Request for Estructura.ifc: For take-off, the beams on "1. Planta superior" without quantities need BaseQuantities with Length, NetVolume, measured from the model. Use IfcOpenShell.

First a look at what the model holds.

```python
import ifcopenshell
import ifcopenshell.util.element
import ifcopenshell.util.unit

model = ifcopenshell.open("Estructura.ifc")
print(model.schema)
for unit_type in ("LENGTHUNIT", "AREAUNIT", "VOLUMEUNIT"):
    print(unit_type, ifcopenshell.util.unit.calculate_unit_scale(model, unit_type))
storey = next(s for s in model.by_type("IfcBuildingStorey") if s.Name == "1. Planta superior")
beams = [e for e in ifcopenshell.util.element.get_decomposition(storey) if e.is_a("IfcBeam")]
for e in sorted(beams, key=lambda e: e.id()):
    print(e.id(), e.is_a(), e.Name, list(ifcopenshell.util.element.get_psets(e, qtos_only=True)), sep=" | ")
```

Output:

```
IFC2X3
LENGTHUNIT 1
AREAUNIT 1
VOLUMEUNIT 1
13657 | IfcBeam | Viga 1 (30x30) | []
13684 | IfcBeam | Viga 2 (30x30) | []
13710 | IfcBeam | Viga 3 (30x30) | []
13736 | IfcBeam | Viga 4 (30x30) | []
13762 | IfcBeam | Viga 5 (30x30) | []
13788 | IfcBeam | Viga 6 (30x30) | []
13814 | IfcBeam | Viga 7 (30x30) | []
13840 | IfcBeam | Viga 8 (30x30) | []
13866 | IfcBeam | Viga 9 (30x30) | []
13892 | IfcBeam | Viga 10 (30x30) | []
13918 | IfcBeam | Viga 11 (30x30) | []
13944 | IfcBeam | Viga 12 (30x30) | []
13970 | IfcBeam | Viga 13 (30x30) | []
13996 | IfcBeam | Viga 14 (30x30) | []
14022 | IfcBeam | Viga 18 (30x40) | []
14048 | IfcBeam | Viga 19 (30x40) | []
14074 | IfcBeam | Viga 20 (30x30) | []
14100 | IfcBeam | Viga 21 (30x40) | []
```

```python
import ifcopenshell
import ifcopenshell.api.pset
import ifcopenshell.geom
import ifcopenshell.util.element
import ifcopenshell.util.shape
import ifcopenshell.util.unit

model = ifcopenshell.open("Estructura.ifc")
unit_scale = ifcopenshell.util.unit.calculate_unit_scale(model)
volume_scale = ifcopenshell.util.unit.calculate_unit_scale(model, "VOLUMEUNIT")
settings = ifcopenshell.geom.settings()

storey = next(s for s in model.by_type("IfcBuildingStorey") if s.Name == "1. Planta superior")
beams = [e for e in ifcopenshell.util.element.get_decomposition(storey) if e.is_a("IfcBeam")]

for e in sorted(beams, key=lambda e: e.id()):
    if ifcopenshell.util.element.get_psets(e, qtos_only=True, should_inherit=False):
        continue
    # Geometry comes back in metres, in the element's own axes.
    shape = ifcopenshell.geom.create_shape(settings, e)
    values = {
        "Length": ifcopenshell.util.shape.get_max_xyz(shape.geometry) / unit_scale,
        "NetVolume": ifcopenshell.util.shape.get_volume(shape.geometry) / volume_scale,
    }
    qto = ifcopenshell.api.pset.add_qto(model, product=e, name="BaseQuantities")
    ifcopenshell.api.pset.edit_qto(model, qto=qto, properties=values)
    print(e.id(), {k: round(v, 3) for k, v in values.items()})

model.write("Estructura_edited.ifc")
```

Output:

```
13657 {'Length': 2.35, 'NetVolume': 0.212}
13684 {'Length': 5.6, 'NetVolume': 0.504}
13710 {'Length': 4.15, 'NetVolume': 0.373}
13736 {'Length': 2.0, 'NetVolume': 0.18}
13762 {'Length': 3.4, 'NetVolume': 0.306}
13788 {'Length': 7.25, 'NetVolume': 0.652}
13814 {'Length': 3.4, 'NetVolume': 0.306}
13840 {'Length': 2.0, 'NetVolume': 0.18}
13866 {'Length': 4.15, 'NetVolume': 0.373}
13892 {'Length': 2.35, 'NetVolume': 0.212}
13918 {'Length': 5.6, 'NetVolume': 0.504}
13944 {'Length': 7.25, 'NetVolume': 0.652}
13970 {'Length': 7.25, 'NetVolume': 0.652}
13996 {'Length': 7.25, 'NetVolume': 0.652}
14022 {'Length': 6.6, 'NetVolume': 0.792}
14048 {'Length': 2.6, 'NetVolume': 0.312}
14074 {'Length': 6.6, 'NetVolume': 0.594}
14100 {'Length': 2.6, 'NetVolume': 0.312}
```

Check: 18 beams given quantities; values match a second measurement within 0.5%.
